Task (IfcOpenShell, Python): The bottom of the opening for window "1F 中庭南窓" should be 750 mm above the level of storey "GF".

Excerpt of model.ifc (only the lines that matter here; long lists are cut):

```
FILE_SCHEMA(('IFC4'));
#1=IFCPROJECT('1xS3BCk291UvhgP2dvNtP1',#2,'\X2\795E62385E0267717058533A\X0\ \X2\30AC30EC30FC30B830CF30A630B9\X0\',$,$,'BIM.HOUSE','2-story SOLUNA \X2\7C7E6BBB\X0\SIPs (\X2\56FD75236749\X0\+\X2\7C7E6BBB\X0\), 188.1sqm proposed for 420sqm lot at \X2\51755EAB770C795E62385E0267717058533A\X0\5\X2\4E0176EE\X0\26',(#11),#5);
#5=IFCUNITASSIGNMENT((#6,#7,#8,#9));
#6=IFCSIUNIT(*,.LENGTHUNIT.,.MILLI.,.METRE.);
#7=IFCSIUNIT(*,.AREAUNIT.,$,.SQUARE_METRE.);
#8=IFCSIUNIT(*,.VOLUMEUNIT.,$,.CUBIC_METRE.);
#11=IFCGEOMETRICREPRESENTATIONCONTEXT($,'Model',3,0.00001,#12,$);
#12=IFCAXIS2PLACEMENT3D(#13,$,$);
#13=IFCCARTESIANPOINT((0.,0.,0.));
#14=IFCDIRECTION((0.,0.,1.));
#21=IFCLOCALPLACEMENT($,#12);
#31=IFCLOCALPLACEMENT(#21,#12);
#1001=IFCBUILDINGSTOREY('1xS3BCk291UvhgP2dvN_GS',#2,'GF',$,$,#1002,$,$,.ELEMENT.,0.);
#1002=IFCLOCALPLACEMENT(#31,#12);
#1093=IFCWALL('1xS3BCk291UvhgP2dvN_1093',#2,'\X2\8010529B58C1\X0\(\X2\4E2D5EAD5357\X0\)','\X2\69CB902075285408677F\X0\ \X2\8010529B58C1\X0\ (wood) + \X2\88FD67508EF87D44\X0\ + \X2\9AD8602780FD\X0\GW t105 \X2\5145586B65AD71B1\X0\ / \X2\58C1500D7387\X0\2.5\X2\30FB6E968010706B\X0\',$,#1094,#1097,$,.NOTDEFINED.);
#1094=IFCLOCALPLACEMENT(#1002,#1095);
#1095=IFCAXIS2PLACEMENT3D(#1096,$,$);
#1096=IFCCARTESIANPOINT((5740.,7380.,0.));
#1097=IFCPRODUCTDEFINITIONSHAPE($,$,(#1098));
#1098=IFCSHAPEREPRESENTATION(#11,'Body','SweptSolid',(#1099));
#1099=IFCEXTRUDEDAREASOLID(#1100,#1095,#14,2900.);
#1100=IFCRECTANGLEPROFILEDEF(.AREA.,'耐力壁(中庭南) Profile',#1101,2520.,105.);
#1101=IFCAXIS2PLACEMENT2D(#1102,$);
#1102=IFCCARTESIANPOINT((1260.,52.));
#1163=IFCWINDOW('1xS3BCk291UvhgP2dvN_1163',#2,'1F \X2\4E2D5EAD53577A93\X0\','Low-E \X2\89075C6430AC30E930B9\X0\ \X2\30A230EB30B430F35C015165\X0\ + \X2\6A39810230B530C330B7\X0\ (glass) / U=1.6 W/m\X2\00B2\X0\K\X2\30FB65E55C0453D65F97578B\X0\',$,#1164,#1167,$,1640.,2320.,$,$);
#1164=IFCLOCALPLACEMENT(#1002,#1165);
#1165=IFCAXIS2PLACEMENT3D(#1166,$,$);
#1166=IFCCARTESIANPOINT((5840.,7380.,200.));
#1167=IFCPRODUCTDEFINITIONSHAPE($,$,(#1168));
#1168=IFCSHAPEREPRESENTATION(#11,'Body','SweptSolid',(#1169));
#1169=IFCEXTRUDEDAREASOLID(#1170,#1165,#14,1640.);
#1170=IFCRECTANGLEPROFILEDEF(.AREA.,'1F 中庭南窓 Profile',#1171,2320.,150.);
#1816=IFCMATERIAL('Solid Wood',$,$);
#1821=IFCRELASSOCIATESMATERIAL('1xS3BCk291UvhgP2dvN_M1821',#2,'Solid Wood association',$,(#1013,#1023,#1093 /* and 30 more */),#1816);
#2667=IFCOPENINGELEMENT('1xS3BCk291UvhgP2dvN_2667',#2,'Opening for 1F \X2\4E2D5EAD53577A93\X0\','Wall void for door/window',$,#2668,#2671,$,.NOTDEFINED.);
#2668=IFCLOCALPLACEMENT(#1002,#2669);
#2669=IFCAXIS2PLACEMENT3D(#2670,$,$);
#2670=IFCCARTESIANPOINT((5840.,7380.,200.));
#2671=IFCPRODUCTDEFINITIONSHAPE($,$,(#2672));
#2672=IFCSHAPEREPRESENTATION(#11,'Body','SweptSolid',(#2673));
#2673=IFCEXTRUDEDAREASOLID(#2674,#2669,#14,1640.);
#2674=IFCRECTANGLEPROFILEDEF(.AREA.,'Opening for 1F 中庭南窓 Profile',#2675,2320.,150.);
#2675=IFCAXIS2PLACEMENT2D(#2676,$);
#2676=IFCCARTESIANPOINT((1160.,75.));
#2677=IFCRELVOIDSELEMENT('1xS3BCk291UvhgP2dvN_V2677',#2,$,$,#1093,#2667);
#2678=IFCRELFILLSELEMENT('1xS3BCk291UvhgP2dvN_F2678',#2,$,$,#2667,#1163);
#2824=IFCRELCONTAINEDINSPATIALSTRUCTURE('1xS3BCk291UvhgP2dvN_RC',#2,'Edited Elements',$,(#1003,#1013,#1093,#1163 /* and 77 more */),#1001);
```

```python
import numpy as np
import ifcopenshell
import ifcopenshell.api.geometry
import ifcopenshell.geom
import ifcopenshell.util.element
import ifcopenshell.util.placement
import ifcopenshell.util.shape
import ifcopenshell.util.unit

model = ifcopenshell.open("model.ifc")
unit_scale = ifcopenshell.util.unit.calculate_unit_scale(model)

window = model.by_guid("1xS3BCk291UvhgP2dvN_1163")
opening = window.FillsVoids[0].RelatingOpeningElement
storey = ifcopenshell.util.element.get_container(window, ifc_class="IfcBuildingStorey")
level = ifcopenshell.util.placement.get_local_placement(storey.ObjectPlacement)[2, 3]

# The opening's origin need not be at the sill, so measure its lowest point.
shape = ifcopenshell.geom.create_shape(ifcopenshell.geom.settings(), opening)
bottom = ifcopenshell.util.shape.get_shape_bottom_elevation(shape, shape.geometry) / unit_scale
dz = level + 750.0 - bottom

shift = np.array([0.0, 0.0, dz])
# The window is not placed relative to its opening, so move both.
for product in (opening, window):
    matrix = ifcopenshell.util.placement.get_local_placement(product.ObjectPlacement)
    matrix[:3, 3] += shift
    ifcopenshell.api.geometry.edit_object_placement(model, product=product, matrix=matrix, is_si=False)

print(f"moved by {dz * unit_scale:+.3f} m")

model.write("model_rev.ifc")
```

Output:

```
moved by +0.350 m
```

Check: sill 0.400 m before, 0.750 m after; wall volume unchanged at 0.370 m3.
